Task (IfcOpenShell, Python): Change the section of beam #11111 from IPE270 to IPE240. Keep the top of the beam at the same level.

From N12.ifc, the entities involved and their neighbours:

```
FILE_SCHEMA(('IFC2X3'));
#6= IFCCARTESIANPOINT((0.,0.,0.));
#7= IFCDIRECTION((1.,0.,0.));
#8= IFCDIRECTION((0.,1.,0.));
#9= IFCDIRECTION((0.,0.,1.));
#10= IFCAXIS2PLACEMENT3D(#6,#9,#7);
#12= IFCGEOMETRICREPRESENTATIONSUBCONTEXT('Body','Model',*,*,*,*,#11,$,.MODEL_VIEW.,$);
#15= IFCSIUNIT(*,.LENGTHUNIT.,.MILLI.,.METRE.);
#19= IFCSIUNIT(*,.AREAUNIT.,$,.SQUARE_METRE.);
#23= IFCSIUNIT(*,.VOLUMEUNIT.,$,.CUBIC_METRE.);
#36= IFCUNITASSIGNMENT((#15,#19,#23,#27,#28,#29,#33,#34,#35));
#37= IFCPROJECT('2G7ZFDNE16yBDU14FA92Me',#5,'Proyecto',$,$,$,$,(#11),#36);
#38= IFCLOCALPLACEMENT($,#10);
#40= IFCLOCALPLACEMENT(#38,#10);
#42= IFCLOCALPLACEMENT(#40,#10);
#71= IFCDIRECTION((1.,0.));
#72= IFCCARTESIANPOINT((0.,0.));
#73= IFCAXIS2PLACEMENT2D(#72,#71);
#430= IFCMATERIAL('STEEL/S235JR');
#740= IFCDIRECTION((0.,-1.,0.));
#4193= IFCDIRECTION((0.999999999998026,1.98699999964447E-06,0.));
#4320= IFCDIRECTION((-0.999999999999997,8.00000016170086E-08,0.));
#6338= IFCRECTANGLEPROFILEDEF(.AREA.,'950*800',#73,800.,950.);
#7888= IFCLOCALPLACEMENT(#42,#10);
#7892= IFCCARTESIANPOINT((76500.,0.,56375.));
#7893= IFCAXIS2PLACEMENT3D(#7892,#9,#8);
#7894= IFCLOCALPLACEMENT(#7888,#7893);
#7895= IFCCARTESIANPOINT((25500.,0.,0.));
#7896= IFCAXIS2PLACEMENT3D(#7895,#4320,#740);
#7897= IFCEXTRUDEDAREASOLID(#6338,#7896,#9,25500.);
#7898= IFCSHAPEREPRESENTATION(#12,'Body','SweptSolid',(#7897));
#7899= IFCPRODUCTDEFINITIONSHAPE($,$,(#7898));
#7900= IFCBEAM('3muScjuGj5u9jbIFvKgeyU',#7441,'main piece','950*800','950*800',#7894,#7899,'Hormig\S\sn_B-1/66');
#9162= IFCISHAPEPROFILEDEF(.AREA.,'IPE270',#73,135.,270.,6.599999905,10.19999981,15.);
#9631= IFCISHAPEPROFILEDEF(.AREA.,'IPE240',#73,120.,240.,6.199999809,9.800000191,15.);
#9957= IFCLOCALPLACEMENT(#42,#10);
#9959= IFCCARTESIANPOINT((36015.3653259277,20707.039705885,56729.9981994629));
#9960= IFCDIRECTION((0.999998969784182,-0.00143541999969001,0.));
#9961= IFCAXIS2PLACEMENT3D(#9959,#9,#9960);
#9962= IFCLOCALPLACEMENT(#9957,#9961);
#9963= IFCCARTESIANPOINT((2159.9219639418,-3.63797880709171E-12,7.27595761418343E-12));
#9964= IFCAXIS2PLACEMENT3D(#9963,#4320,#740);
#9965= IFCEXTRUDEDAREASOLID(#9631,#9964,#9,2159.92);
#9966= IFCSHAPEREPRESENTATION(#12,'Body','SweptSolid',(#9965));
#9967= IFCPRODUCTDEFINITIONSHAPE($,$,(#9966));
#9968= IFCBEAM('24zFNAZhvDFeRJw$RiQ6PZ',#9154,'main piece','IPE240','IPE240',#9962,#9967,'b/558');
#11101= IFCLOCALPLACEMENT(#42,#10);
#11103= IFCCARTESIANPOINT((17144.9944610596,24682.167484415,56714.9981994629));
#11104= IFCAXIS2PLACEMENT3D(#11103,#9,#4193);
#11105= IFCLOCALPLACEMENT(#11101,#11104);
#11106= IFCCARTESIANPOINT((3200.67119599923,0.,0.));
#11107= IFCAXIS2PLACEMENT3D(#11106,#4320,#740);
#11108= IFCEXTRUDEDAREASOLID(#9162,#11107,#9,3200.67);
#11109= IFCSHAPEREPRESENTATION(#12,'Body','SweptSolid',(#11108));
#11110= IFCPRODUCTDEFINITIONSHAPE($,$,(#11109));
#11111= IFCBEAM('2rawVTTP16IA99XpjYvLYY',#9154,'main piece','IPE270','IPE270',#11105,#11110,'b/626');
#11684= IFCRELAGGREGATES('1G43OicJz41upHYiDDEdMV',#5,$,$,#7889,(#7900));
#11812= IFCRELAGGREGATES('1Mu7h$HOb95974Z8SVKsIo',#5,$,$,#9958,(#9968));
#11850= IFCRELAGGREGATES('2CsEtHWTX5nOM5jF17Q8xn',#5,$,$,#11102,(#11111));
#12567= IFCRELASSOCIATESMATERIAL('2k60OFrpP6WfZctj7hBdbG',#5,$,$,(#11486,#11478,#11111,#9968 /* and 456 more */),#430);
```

```python
import ifcopenshell
import ifcopenshell.util.element
import ifcopenshell.util.representation

model = ifcopenshell.open("N12.ifc")

member = model.by_id(11111)
source = next(p for p in model.by_type("IfcIShapeProfileDef") if p.ProfileName == "IPE240")

body = ifcopenshell.util.representation.get_representation(member, "Model", "Body")
solid = body.Items[0]
old_profile = solid.SweptArea

# Copy the section's sizes but keep this member's own profile position.
profile = ifcopenshell.util.element.copy(model, source)
# Profiles are centred, so shift by half the change in depth to hold the top.
shift = (old_profile.OverallDepth - profile.OverallDepth) / 2
x, y = old_profile.Position.Location.Coordinates
up = (0.0, 1.0)  # upwards, in the solid's own plane
location = model.createIfcCartesianPoint((x + up[0] * shift, y + up[1] * shift))
profile.Position = model.createIfcAxis2Placement2D(location, old_profile.Position.RefDirection)
solid.SweptArea = profile
if not model.get_total_inverses(old_profile):
    ifcopenshell.util.element.remove_deep2(model, old_profile)
member.Description = member.Description.replace("IPE270", "IPE240")
member.ObjectType = member.ObjectType.replace("IPE270", "IPE240")

print(solid.SweptArea)

model.write("N12_v2.ifc")
```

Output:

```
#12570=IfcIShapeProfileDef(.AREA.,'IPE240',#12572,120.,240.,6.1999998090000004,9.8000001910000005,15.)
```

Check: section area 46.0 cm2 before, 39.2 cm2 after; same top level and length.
